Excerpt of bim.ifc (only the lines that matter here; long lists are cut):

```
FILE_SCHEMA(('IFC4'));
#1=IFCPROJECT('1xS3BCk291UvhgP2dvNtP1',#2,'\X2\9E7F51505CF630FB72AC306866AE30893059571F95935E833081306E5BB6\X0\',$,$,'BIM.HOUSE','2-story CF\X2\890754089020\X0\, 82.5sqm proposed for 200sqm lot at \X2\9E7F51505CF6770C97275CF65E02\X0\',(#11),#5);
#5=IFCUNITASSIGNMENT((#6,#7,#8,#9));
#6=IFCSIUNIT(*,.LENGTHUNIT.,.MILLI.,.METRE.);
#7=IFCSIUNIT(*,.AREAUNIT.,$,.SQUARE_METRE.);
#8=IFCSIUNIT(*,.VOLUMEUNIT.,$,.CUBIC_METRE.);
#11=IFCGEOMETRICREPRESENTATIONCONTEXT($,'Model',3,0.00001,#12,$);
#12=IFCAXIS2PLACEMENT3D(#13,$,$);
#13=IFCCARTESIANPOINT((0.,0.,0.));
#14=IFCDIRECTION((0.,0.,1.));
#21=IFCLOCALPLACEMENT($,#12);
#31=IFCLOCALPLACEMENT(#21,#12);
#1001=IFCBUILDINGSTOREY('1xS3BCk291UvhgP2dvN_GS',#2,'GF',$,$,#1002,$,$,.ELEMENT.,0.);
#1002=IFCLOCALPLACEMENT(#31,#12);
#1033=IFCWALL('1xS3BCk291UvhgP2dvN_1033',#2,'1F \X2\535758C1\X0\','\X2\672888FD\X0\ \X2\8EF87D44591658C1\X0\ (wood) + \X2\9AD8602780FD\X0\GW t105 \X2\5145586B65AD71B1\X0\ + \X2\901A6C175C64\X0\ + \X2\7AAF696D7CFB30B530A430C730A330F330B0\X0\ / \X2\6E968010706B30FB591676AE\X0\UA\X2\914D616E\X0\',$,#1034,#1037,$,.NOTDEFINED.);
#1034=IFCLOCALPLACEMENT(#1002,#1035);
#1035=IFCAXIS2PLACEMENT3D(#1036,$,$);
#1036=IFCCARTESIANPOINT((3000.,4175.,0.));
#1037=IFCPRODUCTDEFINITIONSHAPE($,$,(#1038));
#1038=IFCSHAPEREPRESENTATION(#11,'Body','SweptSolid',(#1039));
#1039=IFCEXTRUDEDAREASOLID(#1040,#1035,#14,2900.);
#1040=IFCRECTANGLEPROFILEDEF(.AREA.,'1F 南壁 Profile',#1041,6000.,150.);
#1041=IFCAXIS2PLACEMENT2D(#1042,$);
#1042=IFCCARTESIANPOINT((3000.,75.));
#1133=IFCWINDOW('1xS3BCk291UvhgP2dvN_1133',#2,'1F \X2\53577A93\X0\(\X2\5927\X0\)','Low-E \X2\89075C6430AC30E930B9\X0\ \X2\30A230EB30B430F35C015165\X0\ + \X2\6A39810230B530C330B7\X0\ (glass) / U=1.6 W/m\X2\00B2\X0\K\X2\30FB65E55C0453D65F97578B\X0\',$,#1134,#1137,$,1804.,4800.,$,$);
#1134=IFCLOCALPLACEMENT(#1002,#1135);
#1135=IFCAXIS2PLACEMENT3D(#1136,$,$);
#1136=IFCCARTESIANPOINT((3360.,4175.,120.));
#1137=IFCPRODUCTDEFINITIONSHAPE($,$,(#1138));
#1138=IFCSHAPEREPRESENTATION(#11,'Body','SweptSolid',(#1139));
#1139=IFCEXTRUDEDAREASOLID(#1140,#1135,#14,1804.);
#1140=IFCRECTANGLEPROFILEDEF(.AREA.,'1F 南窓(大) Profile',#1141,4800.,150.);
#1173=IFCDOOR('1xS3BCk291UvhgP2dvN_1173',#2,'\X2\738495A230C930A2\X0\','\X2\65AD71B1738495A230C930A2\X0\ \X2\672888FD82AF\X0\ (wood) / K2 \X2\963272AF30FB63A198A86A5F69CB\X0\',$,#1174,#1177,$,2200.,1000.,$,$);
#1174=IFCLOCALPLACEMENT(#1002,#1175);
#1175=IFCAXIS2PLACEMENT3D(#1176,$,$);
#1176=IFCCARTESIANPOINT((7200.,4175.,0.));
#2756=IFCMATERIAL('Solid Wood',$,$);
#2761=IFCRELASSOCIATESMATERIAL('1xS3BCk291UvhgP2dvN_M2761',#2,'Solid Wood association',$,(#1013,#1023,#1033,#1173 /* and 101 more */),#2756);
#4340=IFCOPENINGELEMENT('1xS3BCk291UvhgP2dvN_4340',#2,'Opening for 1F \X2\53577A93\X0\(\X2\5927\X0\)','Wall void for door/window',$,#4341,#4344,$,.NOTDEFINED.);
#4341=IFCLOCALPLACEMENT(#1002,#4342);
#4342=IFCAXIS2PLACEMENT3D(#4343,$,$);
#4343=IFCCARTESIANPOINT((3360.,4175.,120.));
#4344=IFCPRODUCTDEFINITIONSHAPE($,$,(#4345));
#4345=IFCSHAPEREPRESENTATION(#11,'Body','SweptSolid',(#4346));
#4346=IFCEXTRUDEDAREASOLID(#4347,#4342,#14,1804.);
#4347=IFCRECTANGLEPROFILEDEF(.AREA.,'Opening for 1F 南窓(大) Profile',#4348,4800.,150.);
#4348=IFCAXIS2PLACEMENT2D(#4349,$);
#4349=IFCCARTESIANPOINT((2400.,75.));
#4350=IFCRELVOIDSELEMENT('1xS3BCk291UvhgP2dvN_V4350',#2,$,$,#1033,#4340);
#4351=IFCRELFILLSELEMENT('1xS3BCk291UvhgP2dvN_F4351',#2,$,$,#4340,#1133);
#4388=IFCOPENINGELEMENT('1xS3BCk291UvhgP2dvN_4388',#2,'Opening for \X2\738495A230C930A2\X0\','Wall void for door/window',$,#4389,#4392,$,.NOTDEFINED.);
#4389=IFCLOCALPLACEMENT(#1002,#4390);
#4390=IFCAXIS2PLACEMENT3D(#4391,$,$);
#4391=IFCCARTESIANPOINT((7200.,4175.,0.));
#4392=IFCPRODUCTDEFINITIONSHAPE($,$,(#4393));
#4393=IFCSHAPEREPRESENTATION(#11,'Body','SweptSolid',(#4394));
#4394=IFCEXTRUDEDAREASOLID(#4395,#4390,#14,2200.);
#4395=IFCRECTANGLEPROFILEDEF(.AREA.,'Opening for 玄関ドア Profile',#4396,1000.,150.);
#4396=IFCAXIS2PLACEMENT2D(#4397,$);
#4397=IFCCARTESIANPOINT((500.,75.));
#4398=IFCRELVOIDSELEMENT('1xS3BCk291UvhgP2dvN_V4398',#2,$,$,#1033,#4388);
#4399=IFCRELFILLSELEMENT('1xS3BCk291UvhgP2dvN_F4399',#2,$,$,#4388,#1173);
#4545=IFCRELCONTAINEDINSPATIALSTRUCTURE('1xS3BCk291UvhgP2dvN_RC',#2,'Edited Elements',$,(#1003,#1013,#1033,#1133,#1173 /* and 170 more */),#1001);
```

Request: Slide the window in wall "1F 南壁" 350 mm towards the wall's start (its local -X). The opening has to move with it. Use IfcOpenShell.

```python
import ifcopenshell
import ifcopenshell.api.geometry
import ifcopenshell.util.placement
import ifcopenshell.util.unit

model = ifcopenshell.open("bim.ifc")
unit_scale = ifcopenshell.util.unit.calculate_unit_scale(model)

window = model.by_guid("1xS3BCk291UvhgP2dvN_1133")
opening = window.FillsVoids[0].RelatingOpeningElement
wall = opening.VoidsElements[0].RelatingBuildingElement

wall_matrix = ifcopenshell.util.placement.get_local_placement(wall.ObjectPlacement)
shift = wall_matrix[:3, 0] * -0.35 / unit_scale
before = ifcopenshell.util.placement.get_local_placement(window.ObjectPlacement)[:3, 3].copy()

# The window is not placed relative to its opening, so move both.
for product in (opening, window):
    matrix = ifcopenshell.util.placement.get_local_placement(product.ObjectPlacement)
    matrix[:3, 3] += shift
    ifcopenshell.api.geometry.edit_object_placement(model, product=product, matrix=matrix, is_si=False)

after = ifcopenshell.util.placement.get_local_placement(window.ObjectPlacement)[:3, 3]
print("window moved by", (after - before).round(3) + 0.0)

model.write("bim_edited.ifc")
```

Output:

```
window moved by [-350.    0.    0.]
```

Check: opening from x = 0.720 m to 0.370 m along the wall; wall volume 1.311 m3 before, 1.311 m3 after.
